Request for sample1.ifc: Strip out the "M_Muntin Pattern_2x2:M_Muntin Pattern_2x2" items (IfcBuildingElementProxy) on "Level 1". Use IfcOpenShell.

First a look at what the model holds.

```python
import ifcopenshell
import ifcopenshell.util.element

model = ifcopenshell.open("sample1.ifc")
print(model.schema)
storey = next(s for s in model.by_type("IfcBuildingStorey") if s.Name == "Level 1")
proxies = [e for e in ifcopenshell.util.element.get_decomposition(storey) if e.is_a("IfcBuildingElementProxy")]
seen = {}
for e in proxies:
    element_type = ifcopenshell.util.element.get_type(e)
    name = element_type.Name if element_type not in (None, e) else None
    seen[name] = seen.get(name, 0) + 1
for name, count in sorted(seen.items(), key=str):
    print(count, "x", name)
```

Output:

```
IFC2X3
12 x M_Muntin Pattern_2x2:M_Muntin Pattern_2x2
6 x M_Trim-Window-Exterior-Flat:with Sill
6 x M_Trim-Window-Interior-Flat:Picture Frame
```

```python
import ifcopenshell
import ifcopenshell.api.root
import ifcopenshell.util.element

model = ifcopenshell.open("sample1.ifc")

storey = next(s for s in model.by_type("IfcBuildingStorey") if s.Name == "Level 1")
proxies = [e for e in ifcopenshell.util.element.get_decomposition(storey) if e.is_a("IfcBuildingElementProxy")]
targets = [e for e in proxies if (t := ifcopenshell.util.element.get_type(e)) not in (None, e) and t.Name == "M_Muntin Pattern_2x2:M_Muntin Pattern_2x2"]

for e in targets:
    ifcopenshell.api.root.remove_product(model, product=e)
print(len(targets), "removed")

model.write("sample1_edited.ifc")
```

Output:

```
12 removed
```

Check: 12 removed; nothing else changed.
